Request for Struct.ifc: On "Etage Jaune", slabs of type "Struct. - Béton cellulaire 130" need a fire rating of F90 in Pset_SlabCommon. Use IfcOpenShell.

First a look at what the model holds.

```python
import ifcopenshell
import ifcopenshell.util.element

model = ifcopenshell.open("Struct.ifc")
print(model.schema)
storey = next(s for s in model.by_type("IfcBuildingStorey") if s.Name == "Etage Jaune")
slabs = [e for e in ifcopenshell.util.element.get_decomposition(storey) if e.is_a("IfcSlab")]
seen = {}
for e in slabs:
    element_type = ifcopenshell.util.element.get_type(e)
    key = (element_type.Name if element_type != e and element_type else None, ifcopenshell.util.element.get_pset(e, "Pset_SlabCommon", "FireRating"))
    seen[key] = seen.get(key, 0) + 1
for (name, value), count in sorted(seen.items(), key=str):
    print(count, "x", name, "|", value)
```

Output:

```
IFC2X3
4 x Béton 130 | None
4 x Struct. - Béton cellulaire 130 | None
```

```python
import ifcopenshell
import ifcopenshell.api.pset
import ifcopenshell.util.element

model = ifcopenshell.open("Struct.ifc")

storey = next(s for s in model.by_type("IfcBuildingStorey") if s.Name == "Etage Jaune")
slabs = [e for e in ifcopenshell.util.element.get_decomposition(storey) if e.is_a("IfcSlab")]

count = 0
for e in slabs:
    element_type = ifcopenshell.util.element.get_type(e)
    if element_type in (None, e) or element_type.Name != "Struct. - Béton cellulaire 130":
        continue
    # add_pset returns the element's existing set when there is one.
    pset = ifcopenshell.api.pset.add_pset(model, product=e, name="Pset_SlabCommon")
    ifcopenshell.api.pset.edit_pset(model, pset=pset, properties={"FireRating": "F90"})
    count += 1

print(count, "slabs updated")

model.write("Struct_updated.ifc")
```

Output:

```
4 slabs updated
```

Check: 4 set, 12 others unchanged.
